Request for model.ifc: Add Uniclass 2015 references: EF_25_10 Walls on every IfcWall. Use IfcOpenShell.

First a look at what the model holds.

```python
import ifcopenshell

model = ifcopenshell.open("model.ifc")
print(model.schema)
print("classifications:", [c.Name for c in model.by_type("IfcClassification")])
for ifc_class in ("IfcDoor", "IfcRoof", "IfcStair", "IfcWall", "IfcWindow"):
    print(ifc_class, len(model.by_type(ifc_class)))
```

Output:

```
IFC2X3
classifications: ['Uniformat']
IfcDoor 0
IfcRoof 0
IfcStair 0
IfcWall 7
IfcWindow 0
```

```python
import ifcopenshell
import ifcopenshell.api.classification

model = ifcopenshell.open("model.ifc")

# IFC2X3 requires Source and Edition and has no link from the project to the system.
system = model.create_entity("IfcClassification", Source="NBS", Edition="2015", Name="Uniclass 2015")

codes = {
    "IfcWall": ("EF_25_10", "Walls"),
}
for ifc_class, (code, name) in codes.items():
    products = model.by_type(ifc_class)
    ifcopenshell.api.classification.add_reference(
        model, products=products, classification=system, identification=code, name=name
    )
    print(code, len(products))

model.write("model_rev.ifc")
```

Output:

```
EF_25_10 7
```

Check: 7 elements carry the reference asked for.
